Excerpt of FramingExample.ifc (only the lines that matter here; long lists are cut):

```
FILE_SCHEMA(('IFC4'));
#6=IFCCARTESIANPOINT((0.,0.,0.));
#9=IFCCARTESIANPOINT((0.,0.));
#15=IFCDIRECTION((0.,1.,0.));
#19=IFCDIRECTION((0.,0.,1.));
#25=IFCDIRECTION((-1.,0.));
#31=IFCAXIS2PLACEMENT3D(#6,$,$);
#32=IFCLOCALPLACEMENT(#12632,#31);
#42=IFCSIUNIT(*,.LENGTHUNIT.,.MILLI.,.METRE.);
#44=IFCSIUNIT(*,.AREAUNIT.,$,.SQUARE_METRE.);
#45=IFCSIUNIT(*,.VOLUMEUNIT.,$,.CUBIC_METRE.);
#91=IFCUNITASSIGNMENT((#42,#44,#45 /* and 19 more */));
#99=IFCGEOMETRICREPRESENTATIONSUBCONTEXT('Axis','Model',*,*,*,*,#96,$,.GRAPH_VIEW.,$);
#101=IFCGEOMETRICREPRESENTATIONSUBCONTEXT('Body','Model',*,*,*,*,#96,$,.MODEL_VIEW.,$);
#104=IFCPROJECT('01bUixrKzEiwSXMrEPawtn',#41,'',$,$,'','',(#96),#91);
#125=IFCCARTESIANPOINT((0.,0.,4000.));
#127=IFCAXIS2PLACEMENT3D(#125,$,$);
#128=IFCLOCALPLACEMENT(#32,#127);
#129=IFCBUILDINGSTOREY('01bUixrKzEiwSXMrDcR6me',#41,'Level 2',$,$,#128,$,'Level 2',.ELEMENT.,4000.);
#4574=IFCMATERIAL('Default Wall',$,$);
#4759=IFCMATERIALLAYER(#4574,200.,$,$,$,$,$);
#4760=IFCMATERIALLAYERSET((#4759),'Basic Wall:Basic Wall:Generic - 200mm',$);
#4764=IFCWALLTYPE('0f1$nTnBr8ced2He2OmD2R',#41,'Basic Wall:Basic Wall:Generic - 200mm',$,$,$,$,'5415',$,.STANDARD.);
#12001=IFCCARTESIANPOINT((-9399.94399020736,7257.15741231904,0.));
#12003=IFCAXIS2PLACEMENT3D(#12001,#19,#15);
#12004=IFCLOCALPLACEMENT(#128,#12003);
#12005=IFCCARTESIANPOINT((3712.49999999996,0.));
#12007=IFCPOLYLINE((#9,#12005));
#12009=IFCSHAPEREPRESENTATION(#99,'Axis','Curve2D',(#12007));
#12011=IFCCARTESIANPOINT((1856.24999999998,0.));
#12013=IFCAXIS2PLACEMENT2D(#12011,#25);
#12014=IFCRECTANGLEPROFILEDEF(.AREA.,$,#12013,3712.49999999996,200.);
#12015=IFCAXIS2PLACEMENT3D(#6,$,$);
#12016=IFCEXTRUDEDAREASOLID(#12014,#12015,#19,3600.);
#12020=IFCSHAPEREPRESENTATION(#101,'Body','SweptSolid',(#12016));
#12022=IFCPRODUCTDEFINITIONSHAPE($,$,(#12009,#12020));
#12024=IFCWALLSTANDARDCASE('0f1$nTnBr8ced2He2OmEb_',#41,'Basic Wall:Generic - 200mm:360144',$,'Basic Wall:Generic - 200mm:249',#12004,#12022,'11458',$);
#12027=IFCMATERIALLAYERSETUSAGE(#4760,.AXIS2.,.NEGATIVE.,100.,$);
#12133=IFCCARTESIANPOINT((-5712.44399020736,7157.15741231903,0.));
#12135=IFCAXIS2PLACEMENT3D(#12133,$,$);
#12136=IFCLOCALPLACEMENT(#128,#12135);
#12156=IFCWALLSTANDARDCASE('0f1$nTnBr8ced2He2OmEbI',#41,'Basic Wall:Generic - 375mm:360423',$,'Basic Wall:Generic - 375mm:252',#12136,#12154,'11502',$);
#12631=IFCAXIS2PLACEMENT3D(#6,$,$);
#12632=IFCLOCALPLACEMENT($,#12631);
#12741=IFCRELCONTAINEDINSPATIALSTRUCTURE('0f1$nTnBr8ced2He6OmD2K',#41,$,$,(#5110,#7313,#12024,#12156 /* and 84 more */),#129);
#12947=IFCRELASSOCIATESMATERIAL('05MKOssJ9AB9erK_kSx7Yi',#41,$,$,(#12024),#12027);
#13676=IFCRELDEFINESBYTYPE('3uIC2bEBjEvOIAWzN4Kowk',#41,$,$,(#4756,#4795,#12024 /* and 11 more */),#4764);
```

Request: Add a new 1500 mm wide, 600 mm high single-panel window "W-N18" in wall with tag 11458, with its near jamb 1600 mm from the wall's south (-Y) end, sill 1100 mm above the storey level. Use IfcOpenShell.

```python
import numpy as np
import ifcopenshell
import ifcopenshell.api.feature
import ifcopenshell.api.geometry
import ifcopenshell.api.root
import ifcopenshell.api.spatial
import ifcopenshell.geom
import ifcopenshell.util.element
import ifcopenshell.util.placement
import ifcopenshell.util.representation
import ifcopenshell.util.shape
import ifcopenshell.util.unit

model = ifcopenshell.open("FramingExample.ifc")
unit_scale = ifcopenshell.util.unit.calculate_unit_scale(model)
settings = ifcopenshell.geom.settings()


def volume(element):
    """Net volume in cubic metres, openings subtracted."""
    shape = ifcopenshell.geom.create_shape(settings, element)
    return ifcopenshell.util.shape.get_volume(shape.geometry)


wall = model.by_guid("0f1$nTnBr8ced2He2OmEb_")
storey = ifcopenshell.util.element.get_container(wall, ifc_class="IfcBuildingStorey")
context = ifcopenshell.util.representation.get_context(model, "Model", "Body", "MODEL_VIEW")
before = volume(wall)

width, height, from_end, sill = 1.5, 0.6, 1.6, 1.1  # metres

# The wall runs along its own X axis, and the end named is its -X end.
wall_shape = ifcopenshell.geom.create_shape(settings, wall)
x, y, z = ifcopenshell.util.shape.get_vertices(wall_shape.geometry).T
start = x.min() + from_end
face, thickness = float(y.min()), float(y.max() - y.min())
wall_matrix = ifcopenshell.util.placement.get_local_placement(wall.ObjectPlacement)
level = ifcopenshell.util.placement.get_local_placement(storey.ObjectPlacement)[2, 3]


def in_wall(x, y):
    """Placement at x, y metres in the wall's axes, at sill height."""
    matrix = wall_matrix.copy()
    matrix[:, 3] = wall_matrix @ np.array([x / unit_scale, y / unit_scale, 0.0, 1.0])
    matrix[2, 3] = level + sill / unit_scale
    return matrix


# Opening: a box that overshoots both wall faces by 50 mm.
opening = ifcopenshell.api.root.create_entity(model, ifc_class="IfcOpeningElement", predefined_type="OPENING")
box = ifcopenshell.api.geometry.add_wall_representation(
    model, context=context, length=width, height=height, thickness=thickness + 0.1
)
ifcopenshell.api.geometry.assign_representation(model, product=opening, representation=box)
ifcopenshell.api.geometry.edit_object_placement(model, product=opening, matrix=in_wall(start, face - 0.05), is_si=False)
ifcopenshell.api.feature.add_feature(model, feature=opening, element=wall)

window = ifcopenshell.api.root.create_entity(model, ifc_class="IfcWindow", name="W-N18", predefined_type="WINDOW")
window.OverallWidth, window.OverallHeight = width / unit_scale, height / unit_scale
window.PartitioningType = "SINGLE_PANEL"
body = ifcopenshell.api.geometry.add_window_representation(
    model,
    context=context,
    overall_width=window.OverallWidth,
    overall_height=window.OverallHeight,
    partition_type="SINGLE_PANEL",
)
ifcopenshell.api.geometry.assign_representation(model, product=window, representation=body)
ifcopenshell.api.spatial.assign_container(model, products=[window], relating_structure=storey)
ifcopenshell.api.feature.add_filling(model, opening=opening, element=window)

# Centre the window in the wall's thickness.
ifcopenshell.api.geometry.edit_object_placement(model, product=window, matrix=in_wall(start, face), is_si=False)
window_shape = ifcopenshell.geom.create_shape(settings, window)
depth = ifcopenshell.util.shape.get_vertices(window_shape.geometry)[:, 1]
offset = face + thickness / 2 - (depth.min() + depth.max()) / 2
ifcopenshell.api.geometry.edit_object_placement(model, product=window, matrix=in_wall(start, offset), is_si=False)

after = volume(wall)

print(f"wall volume {before:.3f} -> {after:.3f} m3")

model.write("FramingExample_rev.ifc")
```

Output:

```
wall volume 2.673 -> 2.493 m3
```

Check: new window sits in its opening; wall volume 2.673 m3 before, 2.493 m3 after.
